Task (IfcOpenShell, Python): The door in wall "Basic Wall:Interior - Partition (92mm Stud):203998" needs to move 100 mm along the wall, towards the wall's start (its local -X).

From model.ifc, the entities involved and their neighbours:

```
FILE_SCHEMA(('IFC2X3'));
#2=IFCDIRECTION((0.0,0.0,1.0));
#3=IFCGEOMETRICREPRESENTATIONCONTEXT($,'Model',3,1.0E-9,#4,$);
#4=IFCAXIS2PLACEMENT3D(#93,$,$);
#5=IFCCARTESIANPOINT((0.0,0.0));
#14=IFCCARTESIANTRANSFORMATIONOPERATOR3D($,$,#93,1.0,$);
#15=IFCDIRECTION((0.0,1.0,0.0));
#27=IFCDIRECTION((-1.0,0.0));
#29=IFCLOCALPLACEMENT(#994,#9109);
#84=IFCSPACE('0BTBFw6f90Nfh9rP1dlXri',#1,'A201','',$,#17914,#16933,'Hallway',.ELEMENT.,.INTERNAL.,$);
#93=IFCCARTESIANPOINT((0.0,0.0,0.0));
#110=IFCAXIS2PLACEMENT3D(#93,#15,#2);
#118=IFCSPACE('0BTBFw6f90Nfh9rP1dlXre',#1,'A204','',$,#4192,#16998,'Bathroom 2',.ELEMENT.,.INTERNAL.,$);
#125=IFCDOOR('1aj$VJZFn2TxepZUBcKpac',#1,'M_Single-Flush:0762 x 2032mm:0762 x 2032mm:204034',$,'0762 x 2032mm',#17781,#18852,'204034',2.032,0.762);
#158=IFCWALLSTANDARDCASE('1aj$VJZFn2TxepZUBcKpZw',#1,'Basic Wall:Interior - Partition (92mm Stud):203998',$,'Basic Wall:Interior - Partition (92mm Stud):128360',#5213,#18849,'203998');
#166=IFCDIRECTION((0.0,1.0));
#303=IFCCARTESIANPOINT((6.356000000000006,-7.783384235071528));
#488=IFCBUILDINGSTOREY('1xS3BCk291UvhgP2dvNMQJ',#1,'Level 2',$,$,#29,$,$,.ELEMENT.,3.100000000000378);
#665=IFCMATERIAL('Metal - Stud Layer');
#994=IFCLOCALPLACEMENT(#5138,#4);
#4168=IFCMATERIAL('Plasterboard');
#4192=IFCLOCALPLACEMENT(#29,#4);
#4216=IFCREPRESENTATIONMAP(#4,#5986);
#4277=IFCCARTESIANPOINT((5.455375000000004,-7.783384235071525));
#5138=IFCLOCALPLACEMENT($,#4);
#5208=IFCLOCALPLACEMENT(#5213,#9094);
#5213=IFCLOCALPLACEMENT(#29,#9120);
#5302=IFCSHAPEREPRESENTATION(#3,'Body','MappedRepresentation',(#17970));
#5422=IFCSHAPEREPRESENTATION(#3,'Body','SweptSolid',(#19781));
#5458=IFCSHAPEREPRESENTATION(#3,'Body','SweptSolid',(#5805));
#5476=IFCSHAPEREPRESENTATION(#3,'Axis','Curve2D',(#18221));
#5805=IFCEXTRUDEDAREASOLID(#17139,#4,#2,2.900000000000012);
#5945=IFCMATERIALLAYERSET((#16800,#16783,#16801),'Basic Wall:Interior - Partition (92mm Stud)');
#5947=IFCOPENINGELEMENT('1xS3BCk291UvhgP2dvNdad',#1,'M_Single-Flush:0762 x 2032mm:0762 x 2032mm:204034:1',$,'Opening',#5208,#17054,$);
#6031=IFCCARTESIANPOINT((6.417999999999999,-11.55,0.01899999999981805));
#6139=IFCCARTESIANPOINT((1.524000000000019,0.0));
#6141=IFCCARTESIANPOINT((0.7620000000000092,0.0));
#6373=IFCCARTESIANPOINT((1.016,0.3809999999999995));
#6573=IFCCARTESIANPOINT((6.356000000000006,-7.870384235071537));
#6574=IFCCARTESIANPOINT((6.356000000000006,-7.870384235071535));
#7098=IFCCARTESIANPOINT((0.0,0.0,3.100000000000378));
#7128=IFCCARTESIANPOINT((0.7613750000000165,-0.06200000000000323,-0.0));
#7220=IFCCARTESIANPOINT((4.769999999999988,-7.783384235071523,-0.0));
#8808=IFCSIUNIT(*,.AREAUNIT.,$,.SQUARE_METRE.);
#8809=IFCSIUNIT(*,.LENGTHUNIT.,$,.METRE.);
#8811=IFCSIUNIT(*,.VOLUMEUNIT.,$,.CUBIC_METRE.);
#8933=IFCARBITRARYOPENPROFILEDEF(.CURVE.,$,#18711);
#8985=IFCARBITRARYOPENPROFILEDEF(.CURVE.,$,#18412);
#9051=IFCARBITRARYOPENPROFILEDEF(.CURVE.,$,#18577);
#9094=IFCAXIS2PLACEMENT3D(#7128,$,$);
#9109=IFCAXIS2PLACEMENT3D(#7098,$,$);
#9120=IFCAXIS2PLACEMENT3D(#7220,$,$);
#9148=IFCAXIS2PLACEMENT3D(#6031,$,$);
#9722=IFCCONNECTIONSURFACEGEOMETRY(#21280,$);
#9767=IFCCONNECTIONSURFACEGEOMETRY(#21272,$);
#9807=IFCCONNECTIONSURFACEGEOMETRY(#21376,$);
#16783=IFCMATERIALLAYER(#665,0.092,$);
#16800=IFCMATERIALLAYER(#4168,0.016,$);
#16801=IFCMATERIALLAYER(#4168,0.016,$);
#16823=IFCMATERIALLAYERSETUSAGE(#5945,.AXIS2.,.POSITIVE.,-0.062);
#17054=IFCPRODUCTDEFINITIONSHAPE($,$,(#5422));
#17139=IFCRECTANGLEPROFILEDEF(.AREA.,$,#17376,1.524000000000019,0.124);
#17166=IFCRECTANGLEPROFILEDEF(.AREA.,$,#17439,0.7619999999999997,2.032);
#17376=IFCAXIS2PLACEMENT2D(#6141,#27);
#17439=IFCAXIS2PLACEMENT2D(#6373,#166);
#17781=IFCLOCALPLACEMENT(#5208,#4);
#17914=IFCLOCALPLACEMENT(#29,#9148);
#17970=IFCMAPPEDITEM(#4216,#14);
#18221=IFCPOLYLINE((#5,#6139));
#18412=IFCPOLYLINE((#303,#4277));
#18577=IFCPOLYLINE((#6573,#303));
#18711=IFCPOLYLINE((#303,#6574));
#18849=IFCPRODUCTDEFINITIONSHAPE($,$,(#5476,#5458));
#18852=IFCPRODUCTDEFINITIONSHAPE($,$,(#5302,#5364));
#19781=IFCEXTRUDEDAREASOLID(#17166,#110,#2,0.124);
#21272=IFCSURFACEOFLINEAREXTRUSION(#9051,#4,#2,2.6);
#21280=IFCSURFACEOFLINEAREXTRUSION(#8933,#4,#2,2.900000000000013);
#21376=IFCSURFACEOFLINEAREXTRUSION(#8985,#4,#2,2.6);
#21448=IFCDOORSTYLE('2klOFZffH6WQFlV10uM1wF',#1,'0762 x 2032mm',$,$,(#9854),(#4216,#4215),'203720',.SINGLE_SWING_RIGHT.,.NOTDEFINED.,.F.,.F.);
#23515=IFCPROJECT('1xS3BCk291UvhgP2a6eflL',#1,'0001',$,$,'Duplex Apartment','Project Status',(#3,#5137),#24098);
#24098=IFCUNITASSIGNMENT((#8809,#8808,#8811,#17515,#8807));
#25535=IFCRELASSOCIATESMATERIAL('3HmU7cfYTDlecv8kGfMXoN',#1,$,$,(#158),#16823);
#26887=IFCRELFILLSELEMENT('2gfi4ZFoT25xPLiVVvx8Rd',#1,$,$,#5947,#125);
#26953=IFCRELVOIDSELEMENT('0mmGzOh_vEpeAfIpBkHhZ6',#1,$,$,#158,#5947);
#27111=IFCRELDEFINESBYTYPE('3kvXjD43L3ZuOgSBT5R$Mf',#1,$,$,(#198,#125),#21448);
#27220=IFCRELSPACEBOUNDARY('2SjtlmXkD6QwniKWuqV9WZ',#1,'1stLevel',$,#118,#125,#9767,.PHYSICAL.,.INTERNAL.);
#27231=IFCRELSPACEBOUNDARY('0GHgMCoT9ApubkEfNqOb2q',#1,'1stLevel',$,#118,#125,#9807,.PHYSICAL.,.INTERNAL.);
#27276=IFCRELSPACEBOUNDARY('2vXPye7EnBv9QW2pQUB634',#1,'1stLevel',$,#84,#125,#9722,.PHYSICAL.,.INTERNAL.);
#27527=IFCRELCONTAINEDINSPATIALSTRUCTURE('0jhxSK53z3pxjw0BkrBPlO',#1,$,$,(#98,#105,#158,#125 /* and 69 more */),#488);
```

```python
import numpy as np
import ifcopenshell
import ifcopenshell.api.geometry
import ifcopenshell.util.placement
import ifcopenshell.util.unit

model = ifcopenshell.open("model.ifc")
unit_scale = ifcopenshell.util.unit.calculate_unit_scale(model)

door = model.by_guid("1aj$VJZFn2TxepZUBcKpac")
opening = door.FillsVoids[0].RelatingOpeningElement
wall = opening.VoidsElements[0].RelatingBuildingElement

wall_matrix = ifcopenshell.util.placement.get_local_placement(wall.ObjectPlacement)
shift = wall_matrix[:3, 0] * -0.1 / unit_scale
before = ifcopenshell.util.placement.get_local_placement(door.ObjectPlacement)[:3, 3].copy()

# The door is placed relative to its opening, so it follows when the opening moves.
matrix = ifcopenshell.util.placement.get_local_placement(opening.ObjectPlacement)
matrix[:3, 3] += shift
ifcopenshell.api.geometry.edit_object_placement(
    model, product=opening, matrix=matrix, is_si=False, should_transform_children=True
)

# Space boundary surfaces are stored in each space's coordinates; move them too.
for rel in door.ProvidesBoundaries:
    if not rel.ConnectionGeometry:
        continue
    surface = rel.ConnectionGeometry.SurfaceOnRelatingElement
    space_matrix = ifcopenshell.util.placement.get_local_placement(rel.RelatingSpace.ObjectPlacement)
    point = np.array(surface.Position.Location.Coordinates) + space_matrix[:3, :3].T @ shift
    surface.Position = model.createIfcAxis2Placement3D(
        model.createIfcCartesianPoint(point.tolist()), surface.Position.Axis, surface.Position.RefDirection
    )

after = ifcopenshell.util.placement.get_local_placement(door.ObjectPlacement)[:3, 3]
print("door moved by", (after - before).round(3) + 0.0)

model.write("model_rev.ifc")
```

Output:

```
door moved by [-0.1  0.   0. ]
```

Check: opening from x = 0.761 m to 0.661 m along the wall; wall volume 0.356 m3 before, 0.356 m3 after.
